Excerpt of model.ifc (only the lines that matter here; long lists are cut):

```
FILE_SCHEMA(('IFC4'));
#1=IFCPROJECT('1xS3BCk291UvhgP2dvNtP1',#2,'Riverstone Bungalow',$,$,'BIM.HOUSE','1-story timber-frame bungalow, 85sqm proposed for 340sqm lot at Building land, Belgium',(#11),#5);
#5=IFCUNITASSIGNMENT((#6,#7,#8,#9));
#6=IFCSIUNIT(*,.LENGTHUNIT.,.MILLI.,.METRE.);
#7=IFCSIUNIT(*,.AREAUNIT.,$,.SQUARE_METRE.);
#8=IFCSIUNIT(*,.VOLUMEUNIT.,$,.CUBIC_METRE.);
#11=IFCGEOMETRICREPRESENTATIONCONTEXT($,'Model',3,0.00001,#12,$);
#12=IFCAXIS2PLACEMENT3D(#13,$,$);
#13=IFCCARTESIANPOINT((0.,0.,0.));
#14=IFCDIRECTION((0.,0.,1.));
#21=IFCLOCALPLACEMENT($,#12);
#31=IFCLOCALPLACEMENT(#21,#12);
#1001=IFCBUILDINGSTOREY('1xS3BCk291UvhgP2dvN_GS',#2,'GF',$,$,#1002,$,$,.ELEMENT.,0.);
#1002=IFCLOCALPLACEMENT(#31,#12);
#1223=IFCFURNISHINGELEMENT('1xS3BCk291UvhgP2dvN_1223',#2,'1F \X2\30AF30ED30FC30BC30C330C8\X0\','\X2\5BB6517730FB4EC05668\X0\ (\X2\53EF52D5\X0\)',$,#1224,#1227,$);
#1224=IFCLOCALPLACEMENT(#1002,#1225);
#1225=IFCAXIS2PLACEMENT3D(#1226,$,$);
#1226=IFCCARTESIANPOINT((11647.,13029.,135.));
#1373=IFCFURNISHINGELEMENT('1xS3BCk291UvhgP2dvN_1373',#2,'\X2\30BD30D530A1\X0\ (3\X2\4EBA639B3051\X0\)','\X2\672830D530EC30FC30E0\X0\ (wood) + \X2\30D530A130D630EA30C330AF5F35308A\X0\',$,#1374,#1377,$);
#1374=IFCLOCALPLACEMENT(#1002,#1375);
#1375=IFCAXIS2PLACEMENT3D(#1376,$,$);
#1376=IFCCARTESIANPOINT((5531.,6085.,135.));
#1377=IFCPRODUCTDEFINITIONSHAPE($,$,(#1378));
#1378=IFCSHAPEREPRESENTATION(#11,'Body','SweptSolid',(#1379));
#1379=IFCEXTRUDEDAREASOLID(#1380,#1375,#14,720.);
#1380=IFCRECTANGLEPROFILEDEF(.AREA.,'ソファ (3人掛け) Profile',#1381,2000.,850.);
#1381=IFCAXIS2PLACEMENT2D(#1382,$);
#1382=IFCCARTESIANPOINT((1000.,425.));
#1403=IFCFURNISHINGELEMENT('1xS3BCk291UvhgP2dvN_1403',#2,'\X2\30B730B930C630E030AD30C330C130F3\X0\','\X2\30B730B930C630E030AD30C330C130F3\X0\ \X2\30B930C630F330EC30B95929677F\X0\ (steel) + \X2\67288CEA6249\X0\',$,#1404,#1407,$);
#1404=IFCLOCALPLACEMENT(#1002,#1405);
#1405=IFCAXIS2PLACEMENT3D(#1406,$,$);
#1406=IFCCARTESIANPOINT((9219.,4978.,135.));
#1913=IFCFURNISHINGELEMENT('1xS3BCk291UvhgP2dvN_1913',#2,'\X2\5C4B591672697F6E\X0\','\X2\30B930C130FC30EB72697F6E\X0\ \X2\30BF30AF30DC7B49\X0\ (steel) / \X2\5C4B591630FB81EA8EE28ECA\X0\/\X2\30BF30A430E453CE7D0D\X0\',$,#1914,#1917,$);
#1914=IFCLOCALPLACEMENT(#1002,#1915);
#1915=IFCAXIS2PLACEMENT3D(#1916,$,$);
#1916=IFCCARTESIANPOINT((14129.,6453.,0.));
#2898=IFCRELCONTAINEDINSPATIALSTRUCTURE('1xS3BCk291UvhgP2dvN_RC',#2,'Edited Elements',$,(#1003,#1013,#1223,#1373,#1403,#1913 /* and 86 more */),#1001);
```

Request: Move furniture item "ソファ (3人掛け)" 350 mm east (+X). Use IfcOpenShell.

```python
import ifcopenshell
import ifcopenshell.api.geometry
import ifcopenshell.util.placement

model = ifcopenshell.open("model.ifc")

item = model.by_guid("1xS3BCk291UvhgP2dvN_1373")
matrix = ifcopenshell.util.placement.get_local_placement(item.ObjectPlacement)
matrix[0, 3] += 350.0
ifcopenshell.api.geometry.edit_object_placement(model, product=item, matrix=matrix, is_si=False)

print(ifcopenshell.util.placement.get_local_placement(item.ObjectPlacement).round(3) + 0.0)

model.write("model_edited.ifc")
```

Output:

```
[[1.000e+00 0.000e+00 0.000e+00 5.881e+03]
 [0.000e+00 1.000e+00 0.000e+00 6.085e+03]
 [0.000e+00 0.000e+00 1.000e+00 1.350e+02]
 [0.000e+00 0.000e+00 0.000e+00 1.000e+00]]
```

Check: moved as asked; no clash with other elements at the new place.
